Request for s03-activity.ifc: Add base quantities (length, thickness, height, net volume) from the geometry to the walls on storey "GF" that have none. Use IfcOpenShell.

First a look at what the model holds.

```python
import ifcopenshell
import ifcopenshell.util.element
import ifcopenshell.util.unit

model = ifcopenshell.open("s03-activity.ifc")
print(model.schema)
for unit_type in ("LENGTHUNIT", "AREAUNIT", "VOLUMEUNIT"):
    print(unit_type, ifcopenshell.util.unit.calculate_unit_scale(model, unit_type))
storey = next(s for s in model.by_type("IfcBuildingStorey") if s.Name == "GF")
walls = [e for e in ifcopenshell.util.element.get_decomposition(storey) if e.is_a("IfcWall")]
for e in sorted(walls, key=lambda e: e.id()):
    print(e.id(), e.is_a(), e.Name, list(ifcopenshell.util.element.get_psets(e, qtos_only=True)), sep=" | ")
```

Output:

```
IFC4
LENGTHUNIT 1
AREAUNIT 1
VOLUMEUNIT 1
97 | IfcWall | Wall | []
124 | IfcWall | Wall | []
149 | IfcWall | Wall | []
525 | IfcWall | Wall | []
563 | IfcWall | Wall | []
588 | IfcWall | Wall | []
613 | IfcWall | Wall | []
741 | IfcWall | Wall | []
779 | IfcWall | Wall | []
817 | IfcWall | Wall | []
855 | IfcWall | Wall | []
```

```python
import ifcopenshell
import ifcopenshell.api.pset
import ifcopenshell.geom
import ifcopenshell.util.element
import ifcopenshell.util.shape
import ifcopenshell.util.unit

model = ifcopenshell.open("s03-activity.ifc")
unit_scale = ifcopenshell.util.unit.calculate_unit_scale(model)
volume_scale = ifcopenshell.util.unit.calculate_unit_scale(model, "VOLUMEUNIT")
settings = ifcopenshell.geom.settings()

storey = next(s for s in model.by_type("IfcBuildingStorey") if s.Name == "GF")
walls = [e for e in ifcopenshell.util.element.get_decomposition(storey) if e.is_a("IfcWall")]

for e in sorted(walls, key=lambda e: e.id()):
    if ifcopenshell.util.element.get_psets(e, qtos_only=True, should_inherit=False):
        continue
    # Geometry comes back in metres, in the element's own axes.
    shape = ifcopenshell.geom.create_shape(settings, e)
    values = {
        "Length": ifcopenshell.util.shape.get_x(shape.geometry) / unit_scale,
        "Width": ifcopenshell.util.shape.get_y(shape.geometry) / unit_scale,
        "Height": ifcopenshell.util.shape.get_z(shape.geometry) / unit_scale,
        "NetVolume": ifcopenshell.util.shape.get_volume(shape.geometry) / volume_scale,
    }
    qto = ifcopenshell.api.pset.add_qto(model, product=e, name="Qto_WallBaseQuantities")
    ifcopenshell.api.pset.edit_qto(model, qto=qto, properties=values)
    print(e.id(), {k: round(v, 3) for k, v in values.items()})

model.write("s03-activity_updated.ifc")
```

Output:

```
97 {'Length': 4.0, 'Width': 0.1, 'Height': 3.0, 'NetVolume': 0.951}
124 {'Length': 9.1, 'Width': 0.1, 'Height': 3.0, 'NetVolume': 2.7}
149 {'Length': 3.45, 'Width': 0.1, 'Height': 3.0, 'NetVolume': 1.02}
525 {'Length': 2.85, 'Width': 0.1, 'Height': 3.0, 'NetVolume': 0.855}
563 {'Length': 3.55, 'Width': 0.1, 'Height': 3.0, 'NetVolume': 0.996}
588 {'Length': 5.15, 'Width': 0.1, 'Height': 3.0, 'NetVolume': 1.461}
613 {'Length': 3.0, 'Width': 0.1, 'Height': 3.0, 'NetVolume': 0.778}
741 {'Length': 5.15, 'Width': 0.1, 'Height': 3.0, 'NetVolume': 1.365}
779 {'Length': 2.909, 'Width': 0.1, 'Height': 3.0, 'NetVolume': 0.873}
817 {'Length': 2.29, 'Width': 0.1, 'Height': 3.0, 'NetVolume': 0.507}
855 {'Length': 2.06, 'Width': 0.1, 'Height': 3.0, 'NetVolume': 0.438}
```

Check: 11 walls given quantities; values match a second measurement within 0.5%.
